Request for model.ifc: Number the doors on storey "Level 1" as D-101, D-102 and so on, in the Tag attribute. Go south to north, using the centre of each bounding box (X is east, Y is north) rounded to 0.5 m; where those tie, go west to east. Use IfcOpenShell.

First a look at what the model holds.

```python
import ifcopenshell
import ifcopenshell.util.element
import ifcopenshell.util.placement

model = ifcopenshell.open("model.ifc")
print(model.schema)
storey = next(s for s in model.by_type("IfcBuildingStorey") if s.Name == "Level 1")
doors = [e for e in ifcopenshell.util.element.get_decomposition(storey) if e.is_a("IfcDoor")]
for e in sorted(doors, key=lambda e: e.id()):
    origin = ifcopenshell.util.placement.get_local_placement(e.ObjectPlacement)[:3, 3]
    print(e.id(), e.Tag, e.Name, origin.round(2) + 0.0, sep=" | ")
```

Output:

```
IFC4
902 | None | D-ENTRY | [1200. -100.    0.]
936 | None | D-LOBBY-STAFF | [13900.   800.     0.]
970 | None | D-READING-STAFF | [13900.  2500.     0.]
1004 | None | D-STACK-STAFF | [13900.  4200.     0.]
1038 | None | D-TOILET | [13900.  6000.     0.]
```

```python
import ifcopenshell
import ifcopenshell.geom
import ifcopenshell.util.element
import ifcopenshell.util.shape

model = ifcopenshell.open("model.ifc")
settings = ifcopenshell.geom.settings()
settings.set("use-world-coords", True)


def centre(element):
    shape = ifcopenshell.geom.create_shape(settings, element)
    return ifcopenshell.util.shape.get_bbox_centroid(shape.geometry)


storey = next(s for s in model.by_type("IfcBuildingStorey") if s.Name == "Level 1")
doors = [e for e in ifcopenshell.util.element.get_decomposition(storey) if e.is_a("IfcDoor")]

# Insertion points can sit at a corner or the storey origin, so sort by the geometry (in metres).
centres = {e: centre(e) for e in doors}
doors.sort(key=lambda e: (round(centres[e][1] / 0.5), centres[e][0]))

for i, e in enumerate(doors, start=1):
    number = f"D-1{i:02d}"
    e.Tag = number
    print(e.id(), number)

model.write("model-out.ifc")
```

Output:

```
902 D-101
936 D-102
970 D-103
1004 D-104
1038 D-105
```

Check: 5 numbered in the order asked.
